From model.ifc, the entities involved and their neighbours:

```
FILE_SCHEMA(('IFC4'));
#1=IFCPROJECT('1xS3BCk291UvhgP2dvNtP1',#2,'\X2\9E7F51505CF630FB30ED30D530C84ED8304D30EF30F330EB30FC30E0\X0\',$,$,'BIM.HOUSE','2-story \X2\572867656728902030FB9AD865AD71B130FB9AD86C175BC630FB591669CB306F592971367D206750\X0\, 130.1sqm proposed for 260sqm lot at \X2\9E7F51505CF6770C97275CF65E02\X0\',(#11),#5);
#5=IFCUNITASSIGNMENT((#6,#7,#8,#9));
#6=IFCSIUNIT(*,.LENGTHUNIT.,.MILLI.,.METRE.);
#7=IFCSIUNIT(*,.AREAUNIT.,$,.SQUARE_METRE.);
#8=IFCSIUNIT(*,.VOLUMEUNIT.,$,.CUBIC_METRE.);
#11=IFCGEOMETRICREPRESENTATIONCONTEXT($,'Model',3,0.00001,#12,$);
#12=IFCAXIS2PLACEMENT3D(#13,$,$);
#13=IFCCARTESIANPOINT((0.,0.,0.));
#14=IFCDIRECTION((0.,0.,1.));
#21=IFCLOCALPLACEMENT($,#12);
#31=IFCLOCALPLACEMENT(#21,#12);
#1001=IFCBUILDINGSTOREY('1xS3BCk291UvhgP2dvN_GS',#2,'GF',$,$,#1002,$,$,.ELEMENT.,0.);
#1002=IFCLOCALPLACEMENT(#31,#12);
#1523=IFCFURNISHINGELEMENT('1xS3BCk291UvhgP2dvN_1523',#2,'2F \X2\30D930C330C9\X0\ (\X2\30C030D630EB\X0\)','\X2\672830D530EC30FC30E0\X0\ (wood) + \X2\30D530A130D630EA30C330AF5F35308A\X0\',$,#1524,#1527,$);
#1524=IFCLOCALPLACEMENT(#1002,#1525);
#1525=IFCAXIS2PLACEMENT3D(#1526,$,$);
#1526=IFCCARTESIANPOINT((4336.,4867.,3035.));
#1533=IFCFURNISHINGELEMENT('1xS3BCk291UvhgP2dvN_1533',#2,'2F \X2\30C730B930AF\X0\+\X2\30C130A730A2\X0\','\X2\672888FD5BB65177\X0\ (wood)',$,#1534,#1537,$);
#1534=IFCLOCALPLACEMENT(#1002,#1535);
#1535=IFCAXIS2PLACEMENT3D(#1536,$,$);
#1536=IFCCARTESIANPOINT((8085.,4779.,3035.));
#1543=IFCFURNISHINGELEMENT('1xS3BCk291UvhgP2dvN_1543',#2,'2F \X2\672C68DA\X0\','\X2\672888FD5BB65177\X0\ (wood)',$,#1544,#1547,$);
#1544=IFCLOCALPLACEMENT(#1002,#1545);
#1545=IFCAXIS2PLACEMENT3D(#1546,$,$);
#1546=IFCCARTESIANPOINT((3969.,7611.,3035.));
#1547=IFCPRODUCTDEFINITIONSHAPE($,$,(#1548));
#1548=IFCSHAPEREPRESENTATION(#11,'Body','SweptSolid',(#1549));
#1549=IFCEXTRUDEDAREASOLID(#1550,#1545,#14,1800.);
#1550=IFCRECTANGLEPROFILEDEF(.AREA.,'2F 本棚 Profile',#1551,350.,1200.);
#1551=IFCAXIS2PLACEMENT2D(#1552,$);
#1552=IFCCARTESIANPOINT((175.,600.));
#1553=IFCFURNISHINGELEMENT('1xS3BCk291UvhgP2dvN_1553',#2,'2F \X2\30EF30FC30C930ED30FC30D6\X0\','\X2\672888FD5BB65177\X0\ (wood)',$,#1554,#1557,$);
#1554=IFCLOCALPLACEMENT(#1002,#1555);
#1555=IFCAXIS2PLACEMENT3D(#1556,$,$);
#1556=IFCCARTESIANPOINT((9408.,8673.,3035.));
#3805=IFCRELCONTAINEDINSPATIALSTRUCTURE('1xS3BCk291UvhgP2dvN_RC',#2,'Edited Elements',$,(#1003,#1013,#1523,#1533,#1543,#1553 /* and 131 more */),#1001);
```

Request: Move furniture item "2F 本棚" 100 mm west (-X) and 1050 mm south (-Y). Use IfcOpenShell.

```python
import ifcopenshell
import ifcopenshell.api.geometry
import ifcopenshell.util.placement
import ifcopenshell.util.unit

model = ifcopenshell.open("model.ifc")
unit_scale = ifcopenshell.util.unit.calculate_unit_scale(model)

item = model.by_guid("1xS3BCk291UvhgP2dvN_1543")
matrix = ifcopenshell.util.placement.get_local_placement(item.ObjectPlacement)
matrix[0, 3] -= 0.1 / unit_scale
matrix[1, 3] -= 1.05 / unit_scale
ifcopenshell.api.geometry.edit_object_placement(model, product=item, matrix=matrix, is_si=False)

print(ifcopenshell.util.placement.get_local_placement(item.ObjectPlacement).round(3) + 0.0)

model.write("model-out.ifc")
```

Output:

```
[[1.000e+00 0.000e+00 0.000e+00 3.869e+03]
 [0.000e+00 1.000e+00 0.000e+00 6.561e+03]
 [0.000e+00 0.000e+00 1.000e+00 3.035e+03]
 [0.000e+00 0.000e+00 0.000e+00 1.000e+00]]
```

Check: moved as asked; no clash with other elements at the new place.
